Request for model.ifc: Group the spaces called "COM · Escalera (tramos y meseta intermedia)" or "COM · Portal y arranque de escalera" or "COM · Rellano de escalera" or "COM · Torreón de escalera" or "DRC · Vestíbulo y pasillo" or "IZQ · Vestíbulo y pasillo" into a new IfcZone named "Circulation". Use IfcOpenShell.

First a look at what the model holds.

```python
import ifcopenshell

model = ifcopenshell.open("model.ifc")
print(model.schema)
seen = {}
for space in model.by_type("IfcSpace"):
    seen[space.LongName] = seen.get(space.LongName, 0) + 1
for name, count in sorted(seen.items(), key=str):
    print(count, "x", name)
print("zones:", [z.Name for z in model.by_type("IfcZone")][:20])
```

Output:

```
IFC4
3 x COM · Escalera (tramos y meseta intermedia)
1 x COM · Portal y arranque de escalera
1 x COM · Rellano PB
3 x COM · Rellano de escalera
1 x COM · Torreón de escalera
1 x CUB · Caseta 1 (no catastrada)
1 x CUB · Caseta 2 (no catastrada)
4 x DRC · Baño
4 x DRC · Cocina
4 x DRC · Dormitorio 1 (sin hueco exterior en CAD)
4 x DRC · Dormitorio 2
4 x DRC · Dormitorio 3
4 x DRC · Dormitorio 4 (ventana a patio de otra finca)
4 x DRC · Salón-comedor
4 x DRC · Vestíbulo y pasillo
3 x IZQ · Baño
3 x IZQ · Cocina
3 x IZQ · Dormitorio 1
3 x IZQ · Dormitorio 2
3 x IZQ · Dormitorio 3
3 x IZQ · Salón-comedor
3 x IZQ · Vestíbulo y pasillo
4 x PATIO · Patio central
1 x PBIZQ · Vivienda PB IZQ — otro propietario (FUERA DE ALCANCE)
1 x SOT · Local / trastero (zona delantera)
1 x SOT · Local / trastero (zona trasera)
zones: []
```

```python
import ifcopenshell
import ifcopenshell.api.group
import ifcopenshell.api.root

model = ifcopenshell.open("model.ifc")

names = {"COM · Escalera (tramos y meseta intermedia)", "COM · Portal y arranque de escalera", "COM · Rellano de escalera", "COM · Torreón de escalera", "DRC · Vestíbulo y pasillo", "IZQ · Vestíbulo y pasillo"}
spaces = [s for s in model.by_type("IfcSpace") if s.LongName in names]

zone = ifcopenshell.api.root.create_entity(model, ifc_class="IfcZone", name="Circulation")
ifcopenshell.api.group.assign_group(model, products=spaces, group=zone)
print(len(spaces), "spaces in", zone.Name)

model.write("model_edited.ifc")
```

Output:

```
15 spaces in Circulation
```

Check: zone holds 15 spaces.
